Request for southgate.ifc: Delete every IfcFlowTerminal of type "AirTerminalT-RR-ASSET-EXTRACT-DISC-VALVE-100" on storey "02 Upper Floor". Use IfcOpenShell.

First a look at what the model holds.

```python
import ifcopenshell
import ifcopenshell.util.element

model = ifcopenshell.open("southgate.ifc")
print(model.schema)
storey = next(s for s in model.by_type("IfcBuildingStorey") if s.Name == "02 Upper Floor")
terminals = [e for e in ifcopenshell.util.element.get_decomposition(storey) if e.is_a("IfcFlowTerminal")]
seen = {}
for e in terminals:
    element_type = ifcopenshell.util.element.get_type(e)
    name = element_type.Name if element_type not in (None, e) else None
    seen[name] = seen.get(name, 0) + 1
for name, count in sorted(seen.items(), key=str):
    print(count, "x", name)
```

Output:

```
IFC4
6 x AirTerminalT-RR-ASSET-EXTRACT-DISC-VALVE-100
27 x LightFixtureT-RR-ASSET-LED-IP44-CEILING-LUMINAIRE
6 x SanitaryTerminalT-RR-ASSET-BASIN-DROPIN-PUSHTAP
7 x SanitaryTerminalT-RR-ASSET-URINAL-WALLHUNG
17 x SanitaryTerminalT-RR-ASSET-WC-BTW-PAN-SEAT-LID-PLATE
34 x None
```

```python
import ifcopenshell
import ifcopenshell.api.root
import ifcopenshell.util.element

model = ifcopenshell.open("southgate.ifc")

storey = next(s for s in model.by_type("IfcBuildingStorey") if s.Name == "02 Upper Floor")
terminals = [e for e in ifcopenshell.util.element.get_decomposition(storey) if e.is_a("IfcFlowTerminal")]
targets = [e for e in terminals if (t := ifcopenshell.util.element.get_type(e)) not in (None, e) and t.Name == "AirTerminalT-RR-ASSET-EXTRACT-DISC-VALVE-100"]

for e in targets:
    ifcopenshell.api.root.remove_product(model, product=e)
print(len(targets), "removed")

model.write("southgate_edited.ifc")
```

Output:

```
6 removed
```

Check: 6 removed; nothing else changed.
